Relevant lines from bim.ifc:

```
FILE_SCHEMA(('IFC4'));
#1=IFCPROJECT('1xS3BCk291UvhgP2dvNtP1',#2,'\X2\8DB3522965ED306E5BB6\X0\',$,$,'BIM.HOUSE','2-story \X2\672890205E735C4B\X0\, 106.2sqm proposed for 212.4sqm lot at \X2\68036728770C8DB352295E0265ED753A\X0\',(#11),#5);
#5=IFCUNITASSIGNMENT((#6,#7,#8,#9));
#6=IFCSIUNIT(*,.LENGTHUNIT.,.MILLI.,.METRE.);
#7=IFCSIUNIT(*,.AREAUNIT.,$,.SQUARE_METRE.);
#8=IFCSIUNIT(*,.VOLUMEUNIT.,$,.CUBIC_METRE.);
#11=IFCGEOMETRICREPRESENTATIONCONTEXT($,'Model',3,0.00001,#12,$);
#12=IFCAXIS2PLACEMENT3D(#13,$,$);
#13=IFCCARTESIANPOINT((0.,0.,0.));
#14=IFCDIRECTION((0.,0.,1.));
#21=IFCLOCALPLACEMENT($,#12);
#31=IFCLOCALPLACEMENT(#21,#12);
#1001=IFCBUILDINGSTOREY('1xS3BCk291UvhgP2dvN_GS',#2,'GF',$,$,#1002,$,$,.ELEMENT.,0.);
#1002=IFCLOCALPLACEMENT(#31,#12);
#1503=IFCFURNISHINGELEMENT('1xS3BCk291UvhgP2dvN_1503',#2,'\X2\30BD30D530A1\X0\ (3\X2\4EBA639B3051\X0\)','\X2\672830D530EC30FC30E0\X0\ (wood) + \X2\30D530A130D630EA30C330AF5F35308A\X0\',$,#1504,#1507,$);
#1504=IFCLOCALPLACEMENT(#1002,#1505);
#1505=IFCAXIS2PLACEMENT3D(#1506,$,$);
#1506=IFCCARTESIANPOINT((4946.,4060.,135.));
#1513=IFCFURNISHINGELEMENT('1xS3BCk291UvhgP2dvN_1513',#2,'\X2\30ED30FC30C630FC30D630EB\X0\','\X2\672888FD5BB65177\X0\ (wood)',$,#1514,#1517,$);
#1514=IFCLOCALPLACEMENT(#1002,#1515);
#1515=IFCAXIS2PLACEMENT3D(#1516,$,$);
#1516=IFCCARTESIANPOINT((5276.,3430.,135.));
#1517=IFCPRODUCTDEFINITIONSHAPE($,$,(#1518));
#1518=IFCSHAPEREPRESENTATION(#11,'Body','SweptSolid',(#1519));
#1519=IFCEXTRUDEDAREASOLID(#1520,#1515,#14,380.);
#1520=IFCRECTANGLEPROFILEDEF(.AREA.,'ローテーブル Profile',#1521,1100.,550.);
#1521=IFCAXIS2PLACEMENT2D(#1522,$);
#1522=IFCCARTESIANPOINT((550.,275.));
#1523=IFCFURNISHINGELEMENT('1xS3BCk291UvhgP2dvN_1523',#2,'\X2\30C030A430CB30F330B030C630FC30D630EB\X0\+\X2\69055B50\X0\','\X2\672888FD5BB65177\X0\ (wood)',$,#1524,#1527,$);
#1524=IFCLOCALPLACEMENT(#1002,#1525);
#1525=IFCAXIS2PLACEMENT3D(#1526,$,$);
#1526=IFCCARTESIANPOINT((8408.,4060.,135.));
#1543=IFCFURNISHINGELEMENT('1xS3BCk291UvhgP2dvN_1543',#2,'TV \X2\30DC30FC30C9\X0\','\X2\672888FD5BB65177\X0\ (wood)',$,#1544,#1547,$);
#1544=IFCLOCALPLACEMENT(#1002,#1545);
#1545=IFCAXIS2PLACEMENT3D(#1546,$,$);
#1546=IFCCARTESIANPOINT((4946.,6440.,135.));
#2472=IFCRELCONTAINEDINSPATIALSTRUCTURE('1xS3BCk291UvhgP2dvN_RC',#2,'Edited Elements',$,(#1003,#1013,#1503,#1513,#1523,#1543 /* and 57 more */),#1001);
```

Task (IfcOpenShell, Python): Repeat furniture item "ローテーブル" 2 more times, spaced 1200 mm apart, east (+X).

```python
import numpy as np
import ifcopenshell
import ifcopenshell.api.geometry
import ifcopenshell.api.root
import ifcopenshell.util.element
import ifcopenshell.util.placement
import ifcopenshell.util.unit

model = ifcopenshell.open("bim.ifc")
unit_scale = ifcopenshell.util.unit.calculate_unit_scale(model)


def reuse_history(source, copy):
    """copy_class also copies each property set's owner history, people and application; keep the originals."""
    for rel in copy.IsDefinedBy:
        if rel.is_a("IfcRelDefinesByProperties") and (history := rel.RelatingPropertyDefinition.OwnerHistory):
            rel.RelatingPropertyDefinition.OwnerHistory = source.OwnerHistory
            ifcopenshell.util.element.remove_deep2(model, history)


source = model.by_guid("1xS3BCk291UvhgP2dvN_1513")
base = ifcopenshell.util.placement.get_local_placement(source.ObjectPlacement)
step = np.array([1.0, 0.0, 0.0]) * 1.2 / unit_scale

for i in range(1, 3):
    copy = ifcopenshell.api.root.copy_class(model, product=source)
    copy.Representation = ifcopenshell.util.element.copy_deep(
        model, source.Representation, exclude=["IfcGeometricRepresentationContext", "IfcRepresentationMap"]
    )
    reuse_history(source, copy)
    matrix = base.copy()
    matrix[:3, 3] += i * step
    print("added at", matrix[:3, 3].round(3) + 0.0)
    ifcopenshell.api.geometry.edit_object_placement(model, product=copy, matrix=matrix, is_si=False)

model.write("bim_edited.ifc")
```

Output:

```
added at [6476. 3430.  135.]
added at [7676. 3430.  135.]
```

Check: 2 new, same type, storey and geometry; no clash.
